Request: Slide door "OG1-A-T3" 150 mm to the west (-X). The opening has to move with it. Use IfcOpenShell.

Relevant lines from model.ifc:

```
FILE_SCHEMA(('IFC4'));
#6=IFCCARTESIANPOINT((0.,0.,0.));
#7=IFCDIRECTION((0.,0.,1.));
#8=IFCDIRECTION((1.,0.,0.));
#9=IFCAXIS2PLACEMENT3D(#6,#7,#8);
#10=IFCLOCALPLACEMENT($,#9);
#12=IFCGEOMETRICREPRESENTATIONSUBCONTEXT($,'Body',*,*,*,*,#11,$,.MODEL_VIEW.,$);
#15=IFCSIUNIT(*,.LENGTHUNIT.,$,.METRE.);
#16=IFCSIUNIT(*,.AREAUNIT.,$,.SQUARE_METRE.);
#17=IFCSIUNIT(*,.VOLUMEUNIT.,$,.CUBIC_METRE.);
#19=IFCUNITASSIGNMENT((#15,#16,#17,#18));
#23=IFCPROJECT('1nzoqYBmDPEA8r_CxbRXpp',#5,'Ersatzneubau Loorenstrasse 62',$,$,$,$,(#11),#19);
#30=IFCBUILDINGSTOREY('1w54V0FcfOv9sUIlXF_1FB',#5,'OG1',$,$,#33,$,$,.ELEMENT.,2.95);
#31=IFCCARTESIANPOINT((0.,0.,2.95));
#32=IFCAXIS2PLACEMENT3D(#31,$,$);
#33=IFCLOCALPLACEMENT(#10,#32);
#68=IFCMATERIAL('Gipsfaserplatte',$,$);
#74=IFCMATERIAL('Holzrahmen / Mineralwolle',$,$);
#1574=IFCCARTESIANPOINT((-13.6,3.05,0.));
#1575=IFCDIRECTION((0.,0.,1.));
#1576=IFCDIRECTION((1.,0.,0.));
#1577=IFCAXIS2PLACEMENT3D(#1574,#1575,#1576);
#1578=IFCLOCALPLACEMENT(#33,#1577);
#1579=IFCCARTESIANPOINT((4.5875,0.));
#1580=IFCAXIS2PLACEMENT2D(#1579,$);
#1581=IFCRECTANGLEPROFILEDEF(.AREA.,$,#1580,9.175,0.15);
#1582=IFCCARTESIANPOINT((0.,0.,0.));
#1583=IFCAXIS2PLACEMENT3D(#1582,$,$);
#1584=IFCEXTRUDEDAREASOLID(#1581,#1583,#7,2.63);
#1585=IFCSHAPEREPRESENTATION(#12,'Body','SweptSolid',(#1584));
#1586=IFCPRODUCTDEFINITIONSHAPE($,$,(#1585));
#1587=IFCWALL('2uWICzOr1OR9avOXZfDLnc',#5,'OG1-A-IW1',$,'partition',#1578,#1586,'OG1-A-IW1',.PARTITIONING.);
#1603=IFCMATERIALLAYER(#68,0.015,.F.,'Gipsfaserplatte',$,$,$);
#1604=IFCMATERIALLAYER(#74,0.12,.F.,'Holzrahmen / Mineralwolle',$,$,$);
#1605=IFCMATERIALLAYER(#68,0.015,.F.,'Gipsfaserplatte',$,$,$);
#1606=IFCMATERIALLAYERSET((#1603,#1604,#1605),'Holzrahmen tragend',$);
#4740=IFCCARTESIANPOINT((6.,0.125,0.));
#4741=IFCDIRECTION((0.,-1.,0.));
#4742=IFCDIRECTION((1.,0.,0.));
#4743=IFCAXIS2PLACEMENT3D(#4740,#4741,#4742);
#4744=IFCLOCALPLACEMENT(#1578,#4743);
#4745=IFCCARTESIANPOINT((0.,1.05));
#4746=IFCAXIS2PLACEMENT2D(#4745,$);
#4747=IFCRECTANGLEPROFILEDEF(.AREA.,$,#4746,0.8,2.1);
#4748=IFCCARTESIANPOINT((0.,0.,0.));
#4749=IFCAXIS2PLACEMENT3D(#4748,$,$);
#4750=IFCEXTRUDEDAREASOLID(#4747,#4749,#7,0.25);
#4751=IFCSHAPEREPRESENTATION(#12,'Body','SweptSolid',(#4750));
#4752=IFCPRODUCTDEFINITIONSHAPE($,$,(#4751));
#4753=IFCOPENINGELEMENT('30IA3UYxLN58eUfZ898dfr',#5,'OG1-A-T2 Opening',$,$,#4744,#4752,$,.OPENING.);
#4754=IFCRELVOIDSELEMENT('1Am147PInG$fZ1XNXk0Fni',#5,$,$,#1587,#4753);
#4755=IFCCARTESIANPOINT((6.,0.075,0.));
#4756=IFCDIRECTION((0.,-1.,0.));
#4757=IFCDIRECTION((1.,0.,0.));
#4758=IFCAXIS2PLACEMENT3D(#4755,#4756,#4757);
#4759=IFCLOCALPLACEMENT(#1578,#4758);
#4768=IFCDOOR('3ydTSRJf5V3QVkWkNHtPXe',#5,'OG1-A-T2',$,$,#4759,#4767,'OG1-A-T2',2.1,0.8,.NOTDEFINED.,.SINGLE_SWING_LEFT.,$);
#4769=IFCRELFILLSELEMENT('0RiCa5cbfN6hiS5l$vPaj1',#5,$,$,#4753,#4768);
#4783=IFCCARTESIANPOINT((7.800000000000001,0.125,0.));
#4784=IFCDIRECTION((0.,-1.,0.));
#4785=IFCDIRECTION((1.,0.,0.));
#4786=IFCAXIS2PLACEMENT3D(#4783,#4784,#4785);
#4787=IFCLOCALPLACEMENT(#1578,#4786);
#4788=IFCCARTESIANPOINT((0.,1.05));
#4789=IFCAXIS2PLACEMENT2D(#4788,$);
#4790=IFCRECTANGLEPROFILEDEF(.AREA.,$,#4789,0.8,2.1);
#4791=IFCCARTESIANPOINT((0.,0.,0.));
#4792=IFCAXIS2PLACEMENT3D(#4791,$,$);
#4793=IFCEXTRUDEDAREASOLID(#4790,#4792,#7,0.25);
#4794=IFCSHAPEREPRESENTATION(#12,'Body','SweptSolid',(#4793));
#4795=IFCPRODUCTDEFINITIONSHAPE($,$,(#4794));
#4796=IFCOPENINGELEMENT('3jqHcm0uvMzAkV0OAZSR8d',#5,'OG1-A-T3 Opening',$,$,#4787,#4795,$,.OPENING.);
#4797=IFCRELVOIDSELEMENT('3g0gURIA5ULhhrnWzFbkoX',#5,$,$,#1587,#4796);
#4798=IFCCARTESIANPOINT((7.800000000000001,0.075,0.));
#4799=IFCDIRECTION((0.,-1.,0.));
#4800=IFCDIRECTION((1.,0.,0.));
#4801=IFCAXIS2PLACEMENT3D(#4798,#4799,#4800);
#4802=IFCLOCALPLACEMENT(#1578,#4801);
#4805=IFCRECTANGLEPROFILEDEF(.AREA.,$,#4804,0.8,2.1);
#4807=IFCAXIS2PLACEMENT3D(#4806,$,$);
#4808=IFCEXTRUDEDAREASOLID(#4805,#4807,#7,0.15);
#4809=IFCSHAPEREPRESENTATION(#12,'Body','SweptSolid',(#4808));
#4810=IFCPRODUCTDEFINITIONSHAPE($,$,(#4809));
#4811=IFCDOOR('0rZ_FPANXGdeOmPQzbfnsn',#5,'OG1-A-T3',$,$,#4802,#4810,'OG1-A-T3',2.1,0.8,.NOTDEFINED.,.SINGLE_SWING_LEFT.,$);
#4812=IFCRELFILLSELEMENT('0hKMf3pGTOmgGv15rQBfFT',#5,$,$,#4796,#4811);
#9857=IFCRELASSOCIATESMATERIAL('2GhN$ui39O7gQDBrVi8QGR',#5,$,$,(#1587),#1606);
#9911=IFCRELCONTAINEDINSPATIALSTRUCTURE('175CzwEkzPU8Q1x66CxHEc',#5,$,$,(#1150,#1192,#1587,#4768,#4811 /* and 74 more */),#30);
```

```python
import ifcopenshell
import ifcopenshell.api.geometry
import ifcopenshell.util.placement

model = ifcopenshell.open("model.ifc")

door = model.by_guid("0rZ_FPANXGdeOmPQzbfnsn")
opening = door.FillsVoids[0].RelatingOpeningElement
wall = opening.VoidsElements[0].RelatingBuildingElement

wall_matrix = ifcopenshell.util.placement.get_local_placement(wall.ObjectPlacement)
shift = wall_matrix[:3, 0] * -0.15
before = ifcopenshell.util.placement.get_local_placement(door.ObjectPlacement)[:3, 3].copy()

# The door is not placed relative to its opening, so move both.
for product in (opening, door):
    matrix = ifcopenshell.util.placement.get_local_placement(product.ObjectPlacement)
    matrix[:3, 3] += shift
    ifcopenshell.api.geometry.edit_object_placement(model, product=product, matrix=matrix, is_si=False)

after = ifcopenshell.util.placement.get_local_placement(door.ObjectPlacement)[:3, 3]
print("door moved by", (after - before).round(3) + 0.0)

model.write("model_edited.ifc")
```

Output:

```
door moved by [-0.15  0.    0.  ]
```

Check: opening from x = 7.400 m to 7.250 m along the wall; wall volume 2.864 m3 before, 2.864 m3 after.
